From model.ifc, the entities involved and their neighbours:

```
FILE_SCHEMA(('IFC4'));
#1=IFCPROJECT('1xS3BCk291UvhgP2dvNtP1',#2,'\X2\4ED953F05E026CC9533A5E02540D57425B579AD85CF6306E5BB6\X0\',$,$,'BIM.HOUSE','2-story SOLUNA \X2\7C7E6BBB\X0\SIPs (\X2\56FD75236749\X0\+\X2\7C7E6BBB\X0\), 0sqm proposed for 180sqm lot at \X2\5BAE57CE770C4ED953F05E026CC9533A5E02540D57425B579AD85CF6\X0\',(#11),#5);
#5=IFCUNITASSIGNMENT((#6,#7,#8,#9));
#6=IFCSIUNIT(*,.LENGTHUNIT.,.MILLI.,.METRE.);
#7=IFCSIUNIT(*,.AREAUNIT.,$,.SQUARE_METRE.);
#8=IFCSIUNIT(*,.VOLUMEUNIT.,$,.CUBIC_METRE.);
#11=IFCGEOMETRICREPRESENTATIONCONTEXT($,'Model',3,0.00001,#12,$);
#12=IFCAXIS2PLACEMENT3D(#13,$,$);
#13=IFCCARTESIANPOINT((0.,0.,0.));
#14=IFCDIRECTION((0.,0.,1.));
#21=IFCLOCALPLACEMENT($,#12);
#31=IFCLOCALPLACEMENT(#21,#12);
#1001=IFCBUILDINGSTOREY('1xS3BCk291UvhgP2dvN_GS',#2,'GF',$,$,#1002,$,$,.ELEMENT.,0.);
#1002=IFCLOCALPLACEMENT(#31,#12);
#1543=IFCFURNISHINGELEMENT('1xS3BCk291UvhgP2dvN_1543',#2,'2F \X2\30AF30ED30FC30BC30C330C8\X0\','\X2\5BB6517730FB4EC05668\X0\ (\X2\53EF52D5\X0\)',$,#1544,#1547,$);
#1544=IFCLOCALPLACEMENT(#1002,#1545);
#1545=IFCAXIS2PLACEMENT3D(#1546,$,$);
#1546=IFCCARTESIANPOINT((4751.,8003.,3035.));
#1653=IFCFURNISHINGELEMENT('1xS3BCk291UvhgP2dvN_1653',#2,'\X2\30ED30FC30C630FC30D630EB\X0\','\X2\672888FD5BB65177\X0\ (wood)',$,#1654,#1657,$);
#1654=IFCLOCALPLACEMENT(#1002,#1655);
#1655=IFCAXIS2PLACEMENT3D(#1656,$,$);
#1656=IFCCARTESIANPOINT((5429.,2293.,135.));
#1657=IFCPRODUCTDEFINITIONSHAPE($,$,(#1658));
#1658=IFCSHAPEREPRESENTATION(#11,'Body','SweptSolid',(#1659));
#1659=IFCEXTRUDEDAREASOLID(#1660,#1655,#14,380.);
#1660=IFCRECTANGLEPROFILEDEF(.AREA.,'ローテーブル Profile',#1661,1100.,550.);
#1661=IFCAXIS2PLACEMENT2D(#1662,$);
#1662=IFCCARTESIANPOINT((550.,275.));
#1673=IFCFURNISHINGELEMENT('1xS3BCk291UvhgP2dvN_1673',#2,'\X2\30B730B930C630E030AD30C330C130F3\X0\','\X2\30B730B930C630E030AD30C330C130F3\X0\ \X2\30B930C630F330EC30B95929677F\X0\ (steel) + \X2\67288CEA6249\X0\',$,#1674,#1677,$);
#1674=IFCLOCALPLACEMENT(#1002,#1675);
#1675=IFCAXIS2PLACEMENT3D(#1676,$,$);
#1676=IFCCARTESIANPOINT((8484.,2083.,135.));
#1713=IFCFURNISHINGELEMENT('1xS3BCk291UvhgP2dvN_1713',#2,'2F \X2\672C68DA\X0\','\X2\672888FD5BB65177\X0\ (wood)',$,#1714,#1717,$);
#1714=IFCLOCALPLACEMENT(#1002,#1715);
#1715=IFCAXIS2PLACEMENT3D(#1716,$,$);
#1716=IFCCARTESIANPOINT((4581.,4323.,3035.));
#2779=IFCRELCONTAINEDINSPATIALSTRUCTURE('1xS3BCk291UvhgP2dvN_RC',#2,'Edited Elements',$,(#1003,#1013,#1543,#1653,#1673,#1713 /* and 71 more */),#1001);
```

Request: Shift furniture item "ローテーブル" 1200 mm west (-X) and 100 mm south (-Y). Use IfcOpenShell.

```python
import ifcopenshell
import ifcopenshell.api.geometry
import ifcopenshell.util.placement

model = ifcopenshell.open("model.ifc")

item = model.by_id(1653)
matrix = ifcopenshell.util.placement.get_local_placement(item.ObjectPlacement)
matrix[0, 3] -= 1200.0
matrix[1, 3] -= 100.0
ifcopenshell.api.geometry.edit_object_placement(model, product=item, matrix=matrix, is_si=False)

print(ifcopenshell.util.placement.get_local_placement(item.ObjectPlacement).round(3) + 0.0)

model.write("model-out.ifc")
```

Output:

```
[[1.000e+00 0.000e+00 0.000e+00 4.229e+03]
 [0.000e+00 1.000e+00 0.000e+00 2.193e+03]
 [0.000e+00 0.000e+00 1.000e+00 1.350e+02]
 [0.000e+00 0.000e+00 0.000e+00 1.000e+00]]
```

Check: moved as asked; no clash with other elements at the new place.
